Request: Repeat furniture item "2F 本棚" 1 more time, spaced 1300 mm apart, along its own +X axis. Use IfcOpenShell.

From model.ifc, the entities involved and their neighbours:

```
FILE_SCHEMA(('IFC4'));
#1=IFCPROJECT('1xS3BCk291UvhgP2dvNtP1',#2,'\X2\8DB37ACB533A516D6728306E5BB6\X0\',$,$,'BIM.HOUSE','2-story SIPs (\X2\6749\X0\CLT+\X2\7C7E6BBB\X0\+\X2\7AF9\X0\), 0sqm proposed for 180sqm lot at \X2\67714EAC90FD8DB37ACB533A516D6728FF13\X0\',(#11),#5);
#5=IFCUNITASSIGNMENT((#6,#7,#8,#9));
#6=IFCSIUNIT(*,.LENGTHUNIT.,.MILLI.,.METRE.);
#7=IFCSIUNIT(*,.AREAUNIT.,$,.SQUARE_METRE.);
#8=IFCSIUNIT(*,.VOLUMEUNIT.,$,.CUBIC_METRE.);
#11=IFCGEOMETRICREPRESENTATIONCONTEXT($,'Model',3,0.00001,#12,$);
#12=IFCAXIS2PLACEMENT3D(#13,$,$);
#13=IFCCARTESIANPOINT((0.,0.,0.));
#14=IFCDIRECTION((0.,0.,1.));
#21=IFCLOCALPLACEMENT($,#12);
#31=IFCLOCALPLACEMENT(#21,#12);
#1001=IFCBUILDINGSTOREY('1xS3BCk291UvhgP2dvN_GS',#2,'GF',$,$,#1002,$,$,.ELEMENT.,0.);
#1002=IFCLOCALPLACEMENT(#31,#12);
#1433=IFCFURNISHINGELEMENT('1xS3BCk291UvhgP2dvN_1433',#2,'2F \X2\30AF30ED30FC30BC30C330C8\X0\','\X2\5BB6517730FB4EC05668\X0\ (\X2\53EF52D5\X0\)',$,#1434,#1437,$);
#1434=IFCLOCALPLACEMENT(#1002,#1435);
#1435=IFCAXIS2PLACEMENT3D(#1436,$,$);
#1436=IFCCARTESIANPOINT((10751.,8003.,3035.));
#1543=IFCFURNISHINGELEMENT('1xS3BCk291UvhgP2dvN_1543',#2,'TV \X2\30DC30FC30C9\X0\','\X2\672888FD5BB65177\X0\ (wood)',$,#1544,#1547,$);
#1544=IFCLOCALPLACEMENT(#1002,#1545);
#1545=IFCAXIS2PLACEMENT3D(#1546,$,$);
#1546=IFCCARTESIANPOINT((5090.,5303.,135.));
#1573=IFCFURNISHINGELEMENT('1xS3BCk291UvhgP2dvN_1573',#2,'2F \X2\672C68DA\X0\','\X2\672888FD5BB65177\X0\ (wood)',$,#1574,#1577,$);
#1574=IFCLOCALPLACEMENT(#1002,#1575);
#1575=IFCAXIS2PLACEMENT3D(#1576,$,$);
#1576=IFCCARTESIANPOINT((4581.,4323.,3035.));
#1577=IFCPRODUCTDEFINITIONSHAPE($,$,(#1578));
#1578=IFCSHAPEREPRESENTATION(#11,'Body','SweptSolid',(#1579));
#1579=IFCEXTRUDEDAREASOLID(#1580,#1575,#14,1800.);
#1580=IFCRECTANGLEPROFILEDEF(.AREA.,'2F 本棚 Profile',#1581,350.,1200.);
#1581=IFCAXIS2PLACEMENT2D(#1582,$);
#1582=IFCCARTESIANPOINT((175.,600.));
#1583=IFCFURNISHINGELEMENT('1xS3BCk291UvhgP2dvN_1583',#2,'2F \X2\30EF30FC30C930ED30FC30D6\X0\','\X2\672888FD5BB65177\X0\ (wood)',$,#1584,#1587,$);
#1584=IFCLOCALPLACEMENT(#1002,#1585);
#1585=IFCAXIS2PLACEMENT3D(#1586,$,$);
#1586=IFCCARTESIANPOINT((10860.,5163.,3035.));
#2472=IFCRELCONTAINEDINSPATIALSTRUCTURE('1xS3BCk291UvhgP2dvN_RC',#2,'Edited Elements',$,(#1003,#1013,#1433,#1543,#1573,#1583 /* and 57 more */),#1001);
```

```python
import ifcopenshell
import ifcopenshell.api.geometry
import ifcopenshell.api.root
import ifcopenshell.util.element
import ifcopenshell.util.placement
import ifcopenshell.util.unit

model = ifcopenshell.open("model.ifc")
unit_scale = ifcopenshell.util.unit.calculate_unit_scale(model)


def reuse_history(source, copy):
    """copy_class also copies each property set's owner history, people and application; keep the originals."""
    for rel in copy.IsDefinedBy:
        if rel.is_a("IfcRelDefinesByProperties") and (history := rel.RelatingPropertyDefinition.OwnerHistory):
            rel.RelatingPropertyDefinition.OwnerHistory = source.OwnerHistory
            ifcopenshell.util.element.remove_deep2(model, history)


source = model.by_guid("1xS3BCk291UvhgP2dvN_1573")
base = ifcopenshell.util.placement.get_local_placement(source.ObjectPlacement)
step = base[:3, 0] * 1.3 / unit_scale

for i in range(1, 2):
    copy = ifcopenshell.api.root.copy_class(model, product=source)
    copy.Representation = ifcopenshell.util.element.copy_deep(
        model, source.Representation, exclude=["IfcGeometricRepresentationContext", "IfcRepresentationMap"]
    )
    reuse_history(source, copy)
    matrix = base.copy()
    matrix[:3, 3] += i * step
    print("added at", matrix[:3, 3].round(3) + 0.0)
    ifcopenshell.api.geometry.edit_object_placement(model, product=copy, matrix=matrix, is_si=False)

model.write("model_v2.ifc")
```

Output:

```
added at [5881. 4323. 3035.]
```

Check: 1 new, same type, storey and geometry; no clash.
